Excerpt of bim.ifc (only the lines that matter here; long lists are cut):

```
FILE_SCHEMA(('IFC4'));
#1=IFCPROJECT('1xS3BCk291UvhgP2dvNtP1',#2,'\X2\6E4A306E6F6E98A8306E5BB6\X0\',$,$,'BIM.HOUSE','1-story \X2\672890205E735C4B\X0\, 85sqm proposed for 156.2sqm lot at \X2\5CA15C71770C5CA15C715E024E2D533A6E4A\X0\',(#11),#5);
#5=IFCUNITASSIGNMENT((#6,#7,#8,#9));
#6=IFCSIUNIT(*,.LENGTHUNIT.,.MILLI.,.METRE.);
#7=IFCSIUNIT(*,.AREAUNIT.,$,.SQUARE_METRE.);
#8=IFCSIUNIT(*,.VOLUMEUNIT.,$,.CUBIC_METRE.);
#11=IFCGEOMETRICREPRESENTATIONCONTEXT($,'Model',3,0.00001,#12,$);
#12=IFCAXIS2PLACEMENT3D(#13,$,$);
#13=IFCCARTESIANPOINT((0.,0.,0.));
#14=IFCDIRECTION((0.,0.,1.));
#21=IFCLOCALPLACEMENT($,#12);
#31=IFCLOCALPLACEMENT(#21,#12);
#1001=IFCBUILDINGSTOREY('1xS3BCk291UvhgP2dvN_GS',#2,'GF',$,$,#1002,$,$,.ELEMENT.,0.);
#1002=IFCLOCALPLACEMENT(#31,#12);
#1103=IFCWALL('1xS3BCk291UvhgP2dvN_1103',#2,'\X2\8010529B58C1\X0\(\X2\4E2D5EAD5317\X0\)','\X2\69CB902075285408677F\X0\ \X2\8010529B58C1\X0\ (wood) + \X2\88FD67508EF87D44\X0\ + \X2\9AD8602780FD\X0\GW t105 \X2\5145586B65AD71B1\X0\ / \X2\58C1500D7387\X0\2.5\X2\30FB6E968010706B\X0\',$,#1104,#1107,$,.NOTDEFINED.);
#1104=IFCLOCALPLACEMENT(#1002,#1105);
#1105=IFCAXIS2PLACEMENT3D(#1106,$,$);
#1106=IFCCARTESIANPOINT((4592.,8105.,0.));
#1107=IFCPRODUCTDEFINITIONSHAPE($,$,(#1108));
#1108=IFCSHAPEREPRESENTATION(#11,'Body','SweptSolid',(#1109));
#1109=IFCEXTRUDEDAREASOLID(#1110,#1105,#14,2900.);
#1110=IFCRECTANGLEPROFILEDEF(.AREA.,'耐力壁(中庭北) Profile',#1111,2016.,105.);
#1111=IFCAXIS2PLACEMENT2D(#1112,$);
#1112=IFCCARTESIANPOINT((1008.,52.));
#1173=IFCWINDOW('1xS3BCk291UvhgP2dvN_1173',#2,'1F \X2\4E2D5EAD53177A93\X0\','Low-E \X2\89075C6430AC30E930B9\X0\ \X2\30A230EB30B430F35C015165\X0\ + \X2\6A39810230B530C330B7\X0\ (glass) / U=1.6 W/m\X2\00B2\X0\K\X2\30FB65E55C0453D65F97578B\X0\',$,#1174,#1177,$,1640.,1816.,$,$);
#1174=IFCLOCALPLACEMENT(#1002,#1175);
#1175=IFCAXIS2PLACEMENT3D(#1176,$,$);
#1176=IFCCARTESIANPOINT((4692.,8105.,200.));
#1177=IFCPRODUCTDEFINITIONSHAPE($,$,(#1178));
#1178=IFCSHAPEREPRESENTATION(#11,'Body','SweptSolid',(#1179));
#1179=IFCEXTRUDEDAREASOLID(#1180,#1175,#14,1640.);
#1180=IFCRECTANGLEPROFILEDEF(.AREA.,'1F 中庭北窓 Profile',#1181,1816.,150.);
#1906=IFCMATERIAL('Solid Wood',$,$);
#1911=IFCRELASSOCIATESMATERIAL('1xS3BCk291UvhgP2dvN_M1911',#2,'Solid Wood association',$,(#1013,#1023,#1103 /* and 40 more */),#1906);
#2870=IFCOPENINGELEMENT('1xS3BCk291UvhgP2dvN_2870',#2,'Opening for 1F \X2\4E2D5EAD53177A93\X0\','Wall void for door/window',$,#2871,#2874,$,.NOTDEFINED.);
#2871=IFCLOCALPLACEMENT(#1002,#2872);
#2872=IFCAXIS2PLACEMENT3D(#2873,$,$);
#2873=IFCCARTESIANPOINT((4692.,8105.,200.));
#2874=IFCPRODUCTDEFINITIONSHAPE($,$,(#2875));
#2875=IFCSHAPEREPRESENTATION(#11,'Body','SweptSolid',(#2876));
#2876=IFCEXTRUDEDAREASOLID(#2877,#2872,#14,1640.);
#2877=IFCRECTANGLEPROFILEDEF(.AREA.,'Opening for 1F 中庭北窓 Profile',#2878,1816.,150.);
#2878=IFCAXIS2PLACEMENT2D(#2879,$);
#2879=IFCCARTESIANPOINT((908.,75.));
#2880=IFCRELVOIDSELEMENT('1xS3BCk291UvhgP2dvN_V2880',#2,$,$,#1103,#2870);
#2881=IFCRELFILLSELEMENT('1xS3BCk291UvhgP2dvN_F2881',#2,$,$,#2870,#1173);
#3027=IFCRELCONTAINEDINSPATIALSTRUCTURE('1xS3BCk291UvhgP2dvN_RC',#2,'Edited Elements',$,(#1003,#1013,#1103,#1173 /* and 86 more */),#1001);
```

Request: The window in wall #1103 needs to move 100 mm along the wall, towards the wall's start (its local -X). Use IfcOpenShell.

```python
import ifcopenshell
import ifcopenshell.api.geometry
import ifcopenshell.util.placement

model = ifcopenshell.open("bim.ifc")

window = model.by_guid("1xS3BCk291UvhgP2dvN_1173")
opening = window.FillsVoids[0].RelatingOpeningElement
wall = opening.VoidsElements[0].RelatingBuildingElement

wall_matrix = ifcopenshell.util.placement.get_local_placement(wall.ObjectPlacement)
shift = wall_matrix[:3, 0] * -100.0
before = ifcopenshell.util.placement.get_local_placement(window.ObjectPlacement)[:3, 3].copy()

# The window is not placed relative to its opening, so move both.
for product in (opening, window):
    matrix = ifcopenshell.util.placement.get_local_placement(product.ObjectPlacement)
    matrix[:3, 3] += shift
    ifcopenshell.api.geometry.edit_object_placement(model, product=product, matrix=matrix, is_si=False)

after = ifcopenshell.util.placement.get_local_placement(window.ObjectPlacement)[:3, 3]
print("window moved by", (after - before).round(3) + 0.0)

model.write("bim_edited.ifc")
```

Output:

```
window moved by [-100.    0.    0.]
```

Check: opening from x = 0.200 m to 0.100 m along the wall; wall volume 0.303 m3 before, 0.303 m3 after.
